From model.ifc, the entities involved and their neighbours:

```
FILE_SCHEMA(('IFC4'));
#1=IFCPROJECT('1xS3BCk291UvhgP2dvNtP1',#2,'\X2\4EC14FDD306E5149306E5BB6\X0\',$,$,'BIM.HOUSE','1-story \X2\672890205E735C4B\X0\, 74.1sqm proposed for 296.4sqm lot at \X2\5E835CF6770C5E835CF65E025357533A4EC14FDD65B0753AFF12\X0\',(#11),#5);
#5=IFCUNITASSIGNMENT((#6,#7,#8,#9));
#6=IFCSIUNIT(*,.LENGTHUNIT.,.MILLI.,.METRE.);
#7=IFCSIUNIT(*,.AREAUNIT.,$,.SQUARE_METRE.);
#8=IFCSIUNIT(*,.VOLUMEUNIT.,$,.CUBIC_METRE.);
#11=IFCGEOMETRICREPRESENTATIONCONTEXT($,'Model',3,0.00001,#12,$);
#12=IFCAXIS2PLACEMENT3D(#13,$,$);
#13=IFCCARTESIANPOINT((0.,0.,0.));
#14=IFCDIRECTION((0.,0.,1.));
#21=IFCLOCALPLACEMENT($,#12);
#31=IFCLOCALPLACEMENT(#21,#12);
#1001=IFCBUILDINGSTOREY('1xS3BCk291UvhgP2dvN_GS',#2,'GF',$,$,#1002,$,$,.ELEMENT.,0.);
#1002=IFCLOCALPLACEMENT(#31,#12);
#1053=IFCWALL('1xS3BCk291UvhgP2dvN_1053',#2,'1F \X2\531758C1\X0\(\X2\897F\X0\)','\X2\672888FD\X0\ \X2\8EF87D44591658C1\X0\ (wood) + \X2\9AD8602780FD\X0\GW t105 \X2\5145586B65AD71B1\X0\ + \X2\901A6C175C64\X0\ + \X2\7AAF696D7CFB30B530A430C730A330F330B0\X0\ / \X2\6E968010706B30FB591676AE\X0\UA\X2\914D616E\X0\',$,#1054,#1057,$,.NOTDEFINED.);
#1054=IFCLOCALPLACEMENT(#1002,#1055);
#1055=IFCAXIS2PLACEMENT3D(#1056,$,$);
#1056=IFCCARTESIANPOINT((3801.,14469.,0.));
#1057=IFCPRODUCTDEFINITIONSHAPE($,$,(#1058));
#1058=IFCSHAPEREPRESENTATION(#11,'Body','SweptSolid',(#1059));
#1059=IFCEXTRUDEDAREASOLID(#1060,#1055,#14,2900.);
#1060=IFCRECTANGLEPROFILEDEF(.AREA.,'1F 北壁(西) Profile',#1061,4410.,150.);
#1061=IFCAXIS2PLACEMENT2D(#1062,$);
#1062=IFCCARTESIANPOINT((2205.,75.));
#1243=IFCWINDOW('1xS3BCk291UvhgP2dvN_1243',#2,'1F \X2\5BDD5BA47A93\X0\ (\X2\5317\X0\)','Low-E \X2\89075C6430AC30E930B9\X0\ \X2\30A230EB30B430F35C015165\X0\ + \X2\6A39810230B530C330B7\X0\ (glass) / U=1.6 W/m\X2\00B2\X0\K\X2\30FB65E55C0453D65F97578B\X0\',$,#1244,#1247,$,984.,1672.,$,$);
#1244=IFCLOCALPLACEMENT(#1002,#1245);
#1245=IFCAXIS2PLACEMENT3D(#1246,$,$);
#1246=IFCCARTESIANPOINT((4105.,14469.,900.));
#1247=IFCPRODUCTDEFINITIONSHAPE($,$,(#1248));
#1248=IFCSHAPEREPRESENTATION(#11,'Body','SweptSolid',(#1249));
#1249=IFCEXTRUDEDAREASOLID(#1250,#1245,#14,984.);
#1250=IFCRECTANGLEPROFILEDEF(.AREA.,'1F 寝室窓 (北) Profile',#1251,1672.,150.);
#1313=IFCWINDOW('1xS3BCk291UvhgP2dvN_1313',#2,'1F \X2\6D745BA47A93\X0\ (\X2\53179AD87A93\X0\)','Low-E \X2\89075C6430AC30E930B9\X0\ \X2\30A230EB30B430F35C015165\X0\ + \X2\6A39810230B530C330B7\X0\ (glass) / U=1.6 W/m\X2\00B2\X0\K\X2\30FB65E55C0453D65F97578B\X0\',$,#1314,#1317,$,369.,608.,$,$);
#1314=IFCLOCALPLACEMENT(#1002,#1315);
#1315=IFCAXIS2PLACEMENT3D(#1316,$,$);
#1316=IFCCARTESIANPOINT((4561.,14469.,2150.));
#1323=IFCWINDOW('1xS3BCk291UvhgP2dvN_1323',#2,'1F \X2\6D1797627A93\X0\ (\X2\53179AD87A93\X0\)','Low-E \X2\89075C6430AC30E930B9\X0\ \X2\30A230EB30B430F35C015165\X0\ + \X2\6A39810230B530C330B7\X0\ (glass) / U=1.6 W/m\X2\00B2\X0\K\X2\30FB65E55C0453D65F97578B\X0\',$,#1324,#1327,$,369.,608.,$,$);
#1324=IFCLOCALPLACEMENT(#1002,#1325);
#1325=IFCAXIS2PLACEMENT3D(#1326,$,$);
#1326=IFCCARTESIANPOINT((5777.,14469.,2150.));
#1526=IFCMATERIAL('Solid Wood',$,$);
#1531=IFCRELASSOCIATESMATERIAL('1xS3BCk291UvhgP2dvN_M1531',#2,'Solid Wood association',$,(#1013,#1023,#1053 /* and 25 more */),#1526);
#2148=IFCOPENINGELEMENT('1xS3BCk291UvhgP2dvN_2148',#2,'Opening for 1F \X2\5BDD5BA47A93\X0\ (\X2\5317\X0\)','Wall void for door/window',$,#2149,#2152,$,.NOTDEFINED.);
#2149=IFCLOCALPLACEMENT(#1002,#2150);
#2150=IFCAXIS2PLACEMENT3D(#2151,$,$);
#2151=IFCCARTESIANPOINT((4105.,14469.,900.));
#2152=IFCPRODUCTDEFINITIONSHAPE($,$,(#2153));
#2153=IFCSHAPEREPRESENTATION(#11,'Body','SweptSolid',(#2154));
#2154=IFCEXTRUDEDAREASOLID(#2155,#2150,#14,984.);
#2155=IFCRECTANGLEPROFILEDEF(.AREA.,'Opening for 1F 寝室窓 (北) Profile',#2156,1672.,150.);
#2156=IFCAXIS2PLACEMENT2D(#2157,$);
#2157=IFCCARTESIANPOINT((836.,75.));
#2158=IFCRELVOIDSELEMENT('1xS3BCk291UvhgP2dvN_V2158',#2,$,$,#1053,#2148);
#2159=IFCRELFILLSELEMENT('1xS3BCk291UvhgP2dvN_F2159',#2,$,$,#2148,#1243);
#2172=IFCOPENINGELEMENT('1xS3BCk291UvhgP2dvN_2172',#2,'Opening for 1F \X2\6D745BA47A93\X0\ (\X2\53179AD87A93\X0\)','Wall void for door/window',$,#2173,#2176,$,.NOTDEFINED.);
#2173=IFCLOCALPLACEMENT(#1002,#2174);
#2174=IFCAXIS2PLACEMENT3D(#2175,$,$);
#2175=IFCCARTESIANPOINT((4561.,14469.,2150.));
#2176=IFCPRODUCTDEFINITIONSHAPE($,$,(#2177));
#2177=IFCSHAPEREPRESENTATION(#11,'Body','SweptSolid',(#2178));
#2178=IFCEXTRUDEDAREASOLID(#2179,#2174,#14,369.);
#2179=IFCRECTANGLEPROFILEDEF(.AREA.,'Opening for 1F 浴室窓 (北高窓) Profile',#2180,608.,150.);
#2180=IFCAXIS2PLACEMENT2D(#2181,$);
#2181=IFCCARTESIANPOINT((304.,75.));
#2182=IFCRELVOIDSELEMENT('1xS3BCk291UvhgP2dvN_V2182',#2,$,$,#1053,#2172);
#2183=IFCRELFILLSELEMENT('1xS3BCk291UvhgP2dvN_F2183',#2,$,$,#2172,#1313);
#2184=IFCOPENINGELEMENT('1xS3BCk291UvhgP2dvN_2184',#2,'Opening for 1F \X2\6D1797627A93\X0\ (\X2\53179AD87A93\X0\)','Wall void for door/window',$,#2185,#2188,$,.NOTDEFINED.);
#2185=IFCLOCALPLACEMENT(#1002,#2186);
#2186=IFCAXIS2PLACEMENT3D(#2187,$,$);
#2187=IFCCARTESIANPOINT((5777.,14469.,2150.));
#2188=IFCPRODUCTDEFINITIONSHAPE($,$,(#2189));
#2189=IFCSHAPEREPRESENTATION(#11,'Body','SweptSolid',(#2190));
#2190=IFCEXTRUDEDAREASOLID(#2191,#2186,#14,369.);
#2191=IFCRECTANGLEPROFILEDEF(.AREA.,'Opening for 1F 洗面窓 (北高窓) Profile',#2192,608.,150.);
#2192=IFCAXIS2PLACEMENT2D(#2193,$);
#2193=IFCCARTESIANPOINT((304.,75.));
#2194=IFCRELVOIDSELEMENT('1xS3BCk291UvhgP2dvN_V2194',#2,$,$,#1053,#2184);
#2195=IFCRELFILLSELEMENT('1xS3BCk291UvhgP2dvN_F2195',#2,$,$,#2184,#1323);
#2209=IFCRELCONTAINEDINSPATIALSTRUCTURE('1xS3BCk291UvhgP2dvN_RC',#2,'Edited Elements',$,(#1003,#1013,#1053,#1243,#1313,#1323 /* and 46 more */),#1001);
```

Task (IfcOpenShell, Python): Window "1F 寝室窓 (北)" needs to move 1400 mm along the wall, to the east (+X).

```python
import ifcopenshell
import ifcopenshell.api.geometry
import ifcopenshell.util.placement
import ifcopenshell.util.unit

model = ifcopenshell.open("model.ifc")
unit_scale = ifcopenshell.util.unit.calculate_unit_scale(model)

window = model.by_guid("1xS3BCk291UvhgP2dvN_1243")
opening = window.FillsVoids[0].RelatingOpeningElement
wall = opening.VoidsElements[0].RelatingBuildingElement

wall_matrix = ifcopenshell.util.placement.get_local_placement(wall.ObjectPlacement)
shift = wall_matrix[:3, 0] * 1.4 / unit_scale
before = ifcopenshell.util.placement.get_local_placement(window.ObjectPlacement)[:3, 3].copy()

# The window is not placed relative to its opening, so move both.
for product in (opening, window):
    matrix = ifcopenshell.util.placement.get_local_placement(product.ObjectPlacement)
    matrix[:3, 3] += shift
    ifcopenshell.api.geometry.edit_object_placement(model, product=product, matrix=matrix, is_si=False)

after = ifcopenshell.util.placement.get_local_placement(window.ObjectPlacement)[:3, 3]
print("window moved by", (after - before).round(3) + 0.0)

model.write("model_edited.ifc")
```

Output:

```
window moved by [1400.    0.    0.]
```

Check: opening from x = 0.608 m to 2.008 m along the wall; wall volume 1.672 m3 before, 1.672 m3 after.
